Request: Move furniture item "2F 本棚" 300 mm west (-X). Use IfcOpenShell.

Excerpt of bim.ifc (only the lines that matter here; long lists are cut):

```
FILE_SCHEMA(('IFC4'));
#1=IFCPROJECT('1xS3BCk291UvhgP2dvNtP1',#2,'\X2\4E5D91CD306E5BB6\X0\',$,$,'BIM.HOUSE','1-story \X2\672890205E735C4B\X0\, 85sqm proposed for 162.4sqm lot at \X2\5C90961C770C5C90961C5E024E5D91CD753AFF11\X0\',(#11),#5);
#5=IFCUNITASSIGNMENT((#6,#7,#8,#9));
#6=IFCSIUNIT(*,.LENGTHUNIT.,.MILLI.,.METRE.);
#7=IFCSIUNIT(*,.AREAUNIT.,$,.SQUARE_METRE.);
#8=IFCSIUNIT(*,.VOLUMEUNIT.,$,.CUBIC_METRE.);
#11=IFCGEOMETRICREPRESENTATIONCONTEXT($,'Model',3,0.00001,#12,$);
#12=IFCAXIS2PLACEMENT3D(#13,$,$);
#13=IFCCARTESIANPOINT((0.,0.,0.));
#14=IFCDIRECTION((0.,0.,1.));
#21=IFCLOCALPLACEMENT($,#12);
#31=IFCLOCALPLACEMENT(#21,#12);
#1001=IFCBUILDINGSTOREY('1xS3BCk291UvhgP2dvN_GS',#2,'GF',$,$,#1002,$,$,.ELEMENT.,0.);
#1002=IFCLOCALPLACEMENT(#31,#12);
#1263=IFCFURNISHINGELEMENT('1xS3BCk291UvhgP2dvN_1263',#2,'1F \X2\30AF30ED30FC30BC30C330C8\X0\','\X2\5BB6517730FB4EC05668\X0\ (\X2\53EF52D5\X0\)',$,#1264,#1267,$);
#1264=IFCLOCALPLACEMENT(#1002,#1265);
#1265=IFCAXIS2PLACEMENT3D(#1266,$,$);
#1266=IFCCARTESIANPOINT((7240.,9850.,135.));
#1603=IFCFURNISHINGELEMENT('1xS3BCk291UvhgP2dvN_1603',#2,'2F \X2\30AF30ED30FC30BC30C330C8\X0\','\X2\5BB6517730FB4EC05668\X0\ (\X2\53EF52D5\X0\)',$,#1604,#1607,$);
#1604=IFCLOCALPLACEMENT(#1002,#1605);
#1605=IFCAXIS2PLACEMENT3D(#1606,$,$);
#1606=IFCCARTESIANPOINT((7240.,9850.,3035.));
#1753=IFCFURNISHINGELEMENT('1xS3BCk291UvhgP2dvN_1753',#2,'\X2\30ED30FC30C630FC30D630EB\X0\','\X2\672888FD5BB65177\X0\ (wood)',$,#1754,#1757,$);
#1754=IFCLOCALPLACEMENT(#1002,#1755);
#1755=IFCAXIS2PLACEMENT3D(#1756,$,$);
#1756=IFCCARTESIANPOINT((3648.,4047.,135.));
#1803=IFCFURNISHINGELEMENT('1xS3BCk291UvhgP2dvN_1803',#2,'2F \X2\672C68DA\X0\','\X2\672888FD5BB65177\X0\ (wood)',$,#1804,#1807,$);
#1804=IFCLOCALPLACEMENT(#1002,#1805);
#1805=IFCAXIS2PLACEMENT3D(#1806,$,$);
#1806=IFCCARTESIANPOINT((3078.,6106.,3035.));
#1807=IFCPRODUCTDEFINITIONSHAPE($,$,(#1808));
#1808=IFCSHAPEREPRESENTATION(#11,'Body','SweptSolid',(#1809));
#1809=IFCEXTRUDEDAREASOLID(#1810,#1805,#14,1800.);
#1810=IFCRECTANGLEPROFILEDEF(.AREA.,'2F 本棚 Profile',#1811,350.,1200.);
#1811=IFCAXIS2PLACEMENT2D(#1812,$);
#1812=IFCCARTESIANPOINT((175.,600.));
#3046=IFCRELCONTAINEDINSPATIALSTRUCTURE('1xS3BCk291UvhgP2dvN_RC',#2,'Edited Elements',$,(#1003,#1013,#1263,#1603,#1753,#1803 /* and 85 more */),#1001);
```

```python
import ifcopenshell
import ifcopenshell.api.geometry
import ifcopenshell.util.placement

model = ifcopenshell.open("bim.ifc")

item = model.by_id(1803)
matrix = ifcopenshell.util.placement.get_local_placement(item.ObjectPlacement)
matrix[0, 3] -= 300.0
ifcopenshell.api.geometry.edit_object_placement(model, product=item, matrix=matrix, is_si=False)

print(ifcopenshell.util.placement.get_local_placement(item.ObjectPlacement).round(3) + 0.0)

model.write("bim_rev.ifc")
```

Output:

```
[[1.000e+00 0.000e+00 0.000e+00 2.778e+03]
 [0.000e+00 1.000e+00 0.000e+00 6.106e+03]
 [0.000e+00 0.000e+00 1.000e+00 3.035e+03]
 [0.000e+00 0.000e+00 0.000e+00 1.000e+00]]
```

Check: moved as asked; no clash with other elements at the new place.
